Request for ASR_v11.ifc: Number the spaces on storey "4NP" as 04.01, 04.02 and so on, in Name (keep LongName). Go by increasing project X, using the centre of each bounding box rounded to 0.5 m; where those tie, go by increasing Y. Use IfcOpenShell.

First a look at what the model holds.

```python
import ifcopenshell
import ifcopenshell.util.element
import ifcopenshell.util.placement

model = ifcopenshell.open("ASR_v11.ifc")
print(model.schema)
storey = next(s for s in model.by_type("IfcBuildingStorey") if s.Name == "4NP")
spaces = [e for e in ifcopenshell.util.element.get_decomposition(storey) if e.is_a("IfcSpace")]
for e in sorted(spaces, key=lambda e: e.id()):
    origin = ifcopenshell.util.placement.get_local_placement(e.ObjectPlacement)[:3, 3]
    print(e.id(), e.Name, e.LongName, origin.round(2) + 0.0, sep=" | ")
```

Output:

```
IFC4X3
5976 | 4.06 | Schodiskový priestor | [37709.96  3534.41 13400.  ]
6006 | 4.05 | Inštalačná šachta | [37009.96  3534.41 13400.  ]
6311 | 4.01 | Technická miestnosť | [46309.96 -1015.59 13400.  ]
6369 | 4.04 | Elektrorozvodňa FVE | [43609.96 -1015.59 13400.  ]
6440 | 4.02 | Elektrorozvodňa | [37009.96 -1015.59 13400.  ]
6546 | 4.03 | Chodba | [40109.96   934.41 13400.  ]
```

```python
import ifcopenshell
import ifcopenshell.geom
import ifcopenshell.util.element
import ifcopenshell.util.shape

model = ifcopenshell.open("ASR_v11.ifc")
settings = ifcopenshell.geom.settings()
settings.set("use-world-coords", True)


def centre(element):
    shape = ifcopenshell.geom.create_shape(settings, element)
    return ifcopenshell.util.shape.get_bbox_centroid(shape.geometry)


storey = next(s for s in model.by_type("IfcBuildingStorey") if s.Name == "4NP")
spaces = [e for e in ifcopenshell.util.element.get_decomposition(storey) if e.is_a("IfcSpace")]

# Insertion points can sit at a corner or the storey origin, so sort by the geometry (in metres).
centres = {e: centre(e) for e in spaces}
spaces.sort(key=lambda e: (round(centres[e][0] / 0.5), centres[e][1]))

for i, e in enumerate(spaces, start=1):
    number = f"04.{i:02d}"
    e.Name = number
    print(e.id(), number)

model.write("ASR_v11_v2.ifc")
```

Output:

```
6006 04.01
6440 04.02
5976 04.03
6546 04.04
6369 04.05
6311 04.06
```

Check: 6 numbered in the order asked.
